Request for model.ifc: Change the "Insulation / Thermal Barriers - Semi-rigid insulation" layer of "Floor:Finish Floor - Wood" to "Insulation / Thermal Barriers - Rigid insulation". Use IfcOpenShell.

First a look at what the model holds.

```python
import ifcopenshell
import ifcopenshell.util.element

model = ifcopenshell.open("model.ifc")
print(model.schema)
for layer_set in model.by_type("IfcMaterialLayerSet"):
    if layer_set.LayerSetName == "Floor:Finish Floor - Wood":
        for layer in layer_set.MaterialLayers:
            print(layer.id(), layer.Material and layer.Material.Name, layer.LayerThickness, sep=" | ")
        print(len(ifcopenshell.util.element.get_elements_by_material(model, layer_set)), "elements and types use it")
print(sorted(m.Name for m in model.by_type("IfcMaterial") if m.Name)[:60])
```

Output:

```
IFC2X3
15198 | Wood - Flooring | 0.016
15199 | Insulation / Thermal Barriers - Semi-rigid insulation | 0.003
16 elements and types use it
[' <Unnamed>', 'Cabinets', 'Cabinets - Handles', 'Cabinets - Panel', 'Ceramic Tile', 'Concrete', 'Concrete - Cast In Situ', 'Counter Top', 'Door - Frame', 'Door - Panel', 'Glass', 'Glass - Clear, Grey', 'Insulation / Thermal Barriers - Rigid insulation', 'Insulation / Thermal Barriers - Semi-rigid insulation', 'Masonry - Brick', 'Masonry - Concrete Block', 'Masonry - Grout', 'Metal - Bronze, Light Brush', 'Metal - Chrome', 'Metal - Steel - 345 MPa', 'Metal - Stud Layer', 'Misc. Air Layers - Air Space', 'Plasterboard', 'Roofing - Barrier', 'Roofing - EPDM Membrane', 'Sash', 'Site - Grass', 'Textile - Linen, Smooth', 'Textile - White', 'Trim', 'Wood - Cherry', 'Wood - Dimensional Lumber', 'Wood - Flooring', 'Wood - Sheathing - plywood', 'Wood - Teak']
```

```python
import ifcopenshell
import ifcopenshell.api.material

model = ifcopenshell.open("model.ifc")

layer_set = next(s for s in model.by_type("IfcMaterialLayerSet") if s.LayerSetName == "Floor:Finish Floor - Wood")
layer = next(l for l in layer_set.MaterialLayers if l.Material and l.Material.Name == "Insulation / Thermal Barriers - Semi-rigid insulation")
material = next(m for m in model.by_type("IfcMaterial") if m.Name == "Insulation / Thermal Barriers - Rigid insulation")

# Point this one layer at the other material; renaming the old one would change it everywhere.
ifcopenshell.api.material.edit_layer(model, layer=layer, attributes={}, material=material)

print([l.Material.Name if l.Material else None for l in layer_set.MaterialLayers])

model.write("model_updated.ifc")
```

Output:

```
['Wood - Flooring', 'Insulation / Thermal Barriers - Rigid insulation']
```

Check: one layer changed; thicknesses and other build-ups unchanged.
